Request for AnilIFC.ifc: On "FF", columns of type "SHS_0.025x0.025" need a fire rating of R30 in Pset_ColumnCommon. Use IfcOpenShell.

First a look at what the model holds.

```python
import ifcopenshell
import ifcopenshell.util.element

model = ifcopenshell.open("AnilIFC.ifc")
print(model.schema)
storey = next(s for s in model.by_type("IfcBuildingStorey") if s.Name == "FF")
columns = [e for e in ifcopenshell.util.element.get_decomposition(storey) if e.is_a("IfcColumn")]
seen = {}
for e in columns:
    element_type = ifcopenshell.util.element.get_type(e)
    key = (element_type.Name if element_type != e and element_type else None, ifcopenshell.util.element.get_pset(e, "Pset_ColumnCommon", "FireRating"))
    seen[key] = seen.get(key, 0) + 1
for (name, value), count in sorted(seen.items(), key=str):
    print(count, "x", name, "|", value)
```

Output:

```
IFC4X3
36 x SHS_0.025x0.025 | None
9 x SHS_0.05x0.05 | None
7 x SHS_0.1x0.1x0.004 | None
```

```python
import ifcopenshell
import ifcopenshell.api.pset
import ifcopenshell.util.element

model = ifcopenshell.open("AnilIFC.ifc")

storey = next(s for s in model.by_type("IfcBuildingStorey") if s.Name == "FF")
columns = [e for e in ifcopenshell.util.element.get_decomposition(storey) if e.is_a("IfcColumn")]

count = 0
for e in columns:
    element_type = ifcopenshell.util.element.get_type(e)
    if element_type in (None, e) or element_type.Name != "SHS_0.025x0.025":
        continue
    # add_pset returns the element's existing set when there is one.
    pset = ifcopenshell.api.pset.add_pset(model, product=e, name="Pset_ColumnCommon")
    ifcopenshell.api.pset.edit_pset(model, pset=pset, properties={"FireRating": "R30"})
    count += 1

print(count, "columns updated")

model.write("AnilIFC_updated.ifc")
```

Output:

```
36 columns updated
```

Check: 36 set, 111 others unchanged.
